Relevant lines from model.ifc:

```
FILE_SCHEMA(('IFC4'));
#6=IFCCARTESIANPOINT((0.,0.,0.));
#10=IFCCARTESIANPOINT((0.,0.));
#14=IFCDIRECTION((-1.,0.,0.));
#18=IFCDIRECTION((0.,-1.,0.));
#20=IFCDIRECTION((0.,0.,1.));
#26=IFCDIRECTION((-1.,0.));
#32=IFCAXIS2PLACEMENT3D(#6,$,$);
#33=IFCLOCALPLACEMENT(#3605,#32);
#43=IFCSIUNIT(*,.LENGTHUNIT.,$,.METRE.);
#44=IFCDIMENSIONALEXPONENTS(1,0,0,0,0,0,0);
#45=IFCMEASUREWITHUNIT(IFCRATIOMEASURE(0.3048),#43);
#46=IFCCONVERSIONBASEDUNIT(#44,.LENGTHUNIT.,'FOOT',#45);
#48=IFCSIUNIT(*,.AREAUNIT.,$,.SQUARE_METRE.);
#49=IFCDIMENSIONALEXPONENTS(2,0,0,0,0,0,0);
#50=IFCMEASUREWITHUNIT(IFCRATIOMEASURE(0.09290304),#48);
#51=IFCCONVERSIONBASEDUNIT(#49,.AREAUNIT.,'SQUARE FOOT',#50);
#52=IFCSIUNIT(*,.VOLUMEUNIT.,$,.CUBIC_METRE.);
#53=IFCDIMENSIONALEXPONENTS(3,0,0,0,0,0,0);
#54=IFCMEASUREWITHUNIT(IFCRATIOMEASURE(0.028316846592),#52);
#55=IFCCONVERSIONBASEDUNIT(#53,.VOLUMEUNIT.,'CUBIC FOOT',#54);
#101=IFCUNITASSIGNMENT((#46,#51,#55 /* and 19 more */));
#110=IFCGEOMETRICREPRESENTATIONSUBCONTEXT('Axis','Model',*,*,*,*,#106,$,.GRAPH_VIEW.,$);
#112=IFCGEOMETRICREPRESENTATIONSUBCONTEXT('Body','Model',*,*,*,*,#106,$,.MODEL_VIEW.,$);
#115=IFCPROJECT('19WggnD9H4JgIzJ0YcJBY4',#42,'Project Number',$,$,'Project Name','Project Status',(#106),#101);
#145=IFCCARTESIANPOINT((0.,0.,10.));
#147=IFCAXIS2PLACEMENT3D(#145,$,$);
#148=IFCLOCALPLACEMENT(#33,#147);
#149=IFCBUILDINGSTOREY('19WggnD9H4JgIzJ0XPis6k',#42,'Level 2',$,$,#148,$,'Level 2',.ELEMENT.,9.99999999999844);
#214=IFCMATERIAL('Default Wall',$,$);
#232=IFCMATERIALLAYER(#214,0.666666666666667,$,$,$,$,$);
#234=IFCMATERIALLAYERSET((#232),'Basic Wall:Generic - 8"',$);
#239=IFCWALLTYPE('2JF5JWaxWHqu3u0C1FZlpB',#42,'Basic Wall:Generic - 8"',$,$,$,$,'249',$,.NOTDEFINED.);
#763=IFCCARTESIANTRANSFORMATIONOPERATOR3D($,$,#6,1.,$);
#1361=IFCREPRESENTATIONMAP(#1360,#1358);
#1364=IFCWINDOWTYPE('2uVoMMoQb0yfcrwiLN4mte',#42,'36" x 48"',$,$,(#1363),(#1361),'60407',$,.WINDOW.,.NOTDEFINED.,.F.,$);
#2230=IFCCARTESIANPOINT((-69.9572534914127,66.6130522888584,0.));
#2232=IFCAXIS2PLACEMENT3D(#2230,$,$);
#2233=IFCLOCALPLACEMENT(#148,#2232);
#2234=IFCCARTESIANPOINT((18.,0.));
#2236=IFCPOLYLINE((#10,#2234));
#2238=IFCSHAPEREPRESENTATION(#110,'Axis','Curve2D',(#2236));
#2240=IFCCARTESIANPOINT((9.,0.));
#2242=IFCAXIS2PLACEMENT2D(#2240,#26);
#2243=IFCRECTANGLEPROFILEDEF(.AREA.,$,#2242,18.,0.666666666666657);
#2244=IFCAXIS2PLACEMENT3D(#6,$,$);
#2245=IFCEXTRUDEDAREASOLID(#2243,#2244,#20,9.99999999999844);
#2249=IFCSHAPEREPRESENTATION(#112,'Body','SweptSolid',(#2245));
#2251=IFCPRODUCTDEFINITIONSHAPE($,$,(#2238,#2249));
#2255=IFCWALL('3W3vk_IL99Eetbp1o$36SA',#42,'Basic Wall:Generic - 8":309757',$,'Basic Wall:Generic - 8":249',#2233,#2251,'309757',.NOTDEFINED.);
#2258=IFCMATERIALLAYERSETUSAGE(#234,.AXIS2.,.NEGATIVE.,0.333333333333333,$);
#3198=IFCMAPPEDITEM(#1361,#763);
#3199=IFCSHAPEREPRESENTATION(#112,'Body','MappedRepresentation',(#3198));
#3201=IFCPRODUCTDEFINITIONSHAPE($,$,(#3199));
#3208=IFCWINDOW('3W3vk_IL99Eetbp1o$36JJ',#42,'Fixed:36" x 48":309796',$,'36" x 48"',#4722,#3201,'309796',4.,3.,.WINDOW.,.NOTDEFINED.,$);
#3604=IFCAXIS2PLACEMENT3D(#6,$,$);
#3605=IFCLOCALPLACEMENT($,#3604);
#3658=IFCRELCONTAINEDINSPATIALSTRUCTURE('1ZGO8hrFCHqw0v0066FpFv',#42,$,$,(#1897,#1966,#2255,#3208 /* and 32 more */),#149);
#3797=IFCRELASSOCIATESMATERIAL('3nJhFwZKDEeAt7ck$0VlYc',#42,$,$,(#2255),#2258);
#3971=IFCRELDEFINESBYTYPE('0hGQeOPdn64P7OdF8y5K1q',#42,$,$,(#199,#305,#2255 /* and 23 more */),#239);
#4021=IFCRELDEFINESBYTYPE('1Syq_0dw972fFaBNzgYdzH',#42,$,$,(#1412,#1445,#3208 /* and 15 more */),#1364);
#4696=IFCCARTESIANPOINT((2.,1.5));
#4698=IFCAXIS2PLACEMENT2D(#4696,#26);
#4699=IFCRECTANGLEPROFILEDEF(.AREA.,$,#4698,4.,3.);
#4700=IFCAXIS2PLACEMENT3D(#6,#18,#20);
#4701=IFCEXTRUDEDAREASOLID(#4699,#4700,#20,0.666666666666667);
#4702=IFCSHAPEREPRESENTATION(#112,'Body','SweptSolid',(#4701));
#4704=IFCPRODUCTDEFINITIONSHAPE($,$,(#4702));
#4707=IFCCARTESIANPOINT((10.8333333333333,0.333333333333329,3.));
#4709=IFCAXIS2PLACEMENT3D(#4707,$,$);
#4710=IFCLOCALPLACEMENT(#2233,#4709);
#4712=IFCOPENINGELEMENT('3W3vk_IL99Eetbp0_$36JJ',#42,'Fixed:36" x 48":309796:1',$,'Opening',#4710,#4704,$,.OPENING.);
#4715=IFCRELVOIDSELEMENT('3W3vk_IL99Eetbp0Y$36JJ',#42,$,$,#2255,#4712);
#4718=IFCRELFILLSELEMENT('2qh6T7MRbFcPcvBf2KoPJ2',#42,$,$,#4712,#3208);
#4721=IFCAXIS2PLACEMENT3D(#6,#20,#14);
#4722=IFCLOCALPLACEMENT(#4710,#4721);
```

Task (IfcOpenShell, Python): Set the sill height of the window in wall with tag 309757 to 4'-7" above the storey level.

```python
import numpy as np
import ifcopenshell
import ifcopenshell.api.geometry
import ifcopenshell.geom
import ifcopenshell.util.element
import ifcopenshell.util.placement
import ifcopenshell.util.shape
import ifcopenshell.util.unit

model = ifcopenshell.open("model.ifc")
unit_scale = ifcopenshell.util.unit.calculate_unit_scale(model)

window = model.by_guid("3W3vk_IL99Eetbp1o$36JJ")
opening = window.FillsVoids[0].RelatingOpeningElement
storey = ifcopenshell.util.element.get_container(window, ifc_class="IfcBuildingStorey")
level = ifcopenshell.util.placement.get_local_placement(storey.ObjectPlacement)[2, 3]

# The opening's origin need not be at the sill, so measure its lowest point.
shape = ifcopenshell.geom.create_shape(ifcopenshell.geom.settings(), opening)
bottom = ifcopenshell.util.shape.get_shape_bottom_elevation(shape, shape.geometry) / unit_scale
dz = level + 55 * 0.0254 / unit_scale - bottom

shift = np.array([0.0, 0.0, dz])
# The window is placed relative to its opening, so it follows when the opening moves.
matrix = ifcopenshell.util.placement.get_local_placement(opening.ObjectPlacement)
matrix[:3, 3] += shift
ifcopenshell.api.geometry.edit_object_placement(
    model, product=opening, matrix=matrix, is_si=False, should_transform_children=True
)

print(f"moved by {dz * unit_scale:+.3f} m")

model.write("model-out.ifc")
```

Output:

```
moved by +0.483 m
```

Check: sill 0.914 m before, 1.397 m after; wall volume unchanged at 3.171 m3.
